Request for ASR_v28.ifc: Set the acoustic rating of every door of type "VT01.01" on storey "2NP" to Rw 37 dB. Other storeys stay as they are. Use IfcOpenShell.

First a look at what the model holds.

```python
import ifcopenshell
import ifcopenshell.util.element

model = ifcopenshell.open("ASR_v28.ifc")
print(model.schema)
storey = next(s for s in model.by_type("IfcBuildingStorey") if s.Name == "2NP")
doors = [e for e in ifcopenshell.util.element.get_decomposition(storey) if e.is_a("IfcDoor")]
seen = {}
for e in doors:
    element_type = ifcopenshell.util.element.get_type(e)
    key = (element_type.Name if element_type != e and element_type else None, ifcopenshell.util.element.get_pset(e, "Pset_DoorCommon", "AcousticRating"))
    seen[key] = seen.get(key, 0) + 1
for (name, value), count in sorted(seen.items(), key=str):
    print(count, "x", name, "|", value)
```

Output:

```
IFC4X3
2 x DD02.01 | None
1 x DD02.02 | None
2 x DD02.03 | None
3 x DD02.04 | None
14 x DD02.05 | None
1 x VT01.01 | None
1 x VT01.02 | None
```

```python
import ifcopenshell
import ifcopenshell.api.pset
import ifcopenshell.util.element

model = ifcopenshell.open("ASR_v28.ifc")

storey = next(s for s in model.by_type("IfcBuildingStorey") if s.Name == "2NP")
doors = [e for e in ifcopenshell.util.element.get_decomposition(storey) if e.is_a("IfcDoor")]

count = 0
for e in doors:
    element_type = ifcopenshell.util.element.get_type(e)
    if element_type in (None, e) or element_type.Name != "VT01.01":
        continue
    # add_pset returns the element's existing set when there is one.
    pset = ifcopenshell.api.pset.add_pset(model, product=e, name="Pset_DoorCommon")
    ifcopenshell.api.pset.edit_pset(model, pset=pset, properties={"AcousticRating": "Rw 37 dB"})
    count += 1

print(count, "doors updated")

model.write("ASR_v28_edited.ifc")
```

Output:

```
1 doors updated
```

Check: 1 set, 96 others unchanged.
